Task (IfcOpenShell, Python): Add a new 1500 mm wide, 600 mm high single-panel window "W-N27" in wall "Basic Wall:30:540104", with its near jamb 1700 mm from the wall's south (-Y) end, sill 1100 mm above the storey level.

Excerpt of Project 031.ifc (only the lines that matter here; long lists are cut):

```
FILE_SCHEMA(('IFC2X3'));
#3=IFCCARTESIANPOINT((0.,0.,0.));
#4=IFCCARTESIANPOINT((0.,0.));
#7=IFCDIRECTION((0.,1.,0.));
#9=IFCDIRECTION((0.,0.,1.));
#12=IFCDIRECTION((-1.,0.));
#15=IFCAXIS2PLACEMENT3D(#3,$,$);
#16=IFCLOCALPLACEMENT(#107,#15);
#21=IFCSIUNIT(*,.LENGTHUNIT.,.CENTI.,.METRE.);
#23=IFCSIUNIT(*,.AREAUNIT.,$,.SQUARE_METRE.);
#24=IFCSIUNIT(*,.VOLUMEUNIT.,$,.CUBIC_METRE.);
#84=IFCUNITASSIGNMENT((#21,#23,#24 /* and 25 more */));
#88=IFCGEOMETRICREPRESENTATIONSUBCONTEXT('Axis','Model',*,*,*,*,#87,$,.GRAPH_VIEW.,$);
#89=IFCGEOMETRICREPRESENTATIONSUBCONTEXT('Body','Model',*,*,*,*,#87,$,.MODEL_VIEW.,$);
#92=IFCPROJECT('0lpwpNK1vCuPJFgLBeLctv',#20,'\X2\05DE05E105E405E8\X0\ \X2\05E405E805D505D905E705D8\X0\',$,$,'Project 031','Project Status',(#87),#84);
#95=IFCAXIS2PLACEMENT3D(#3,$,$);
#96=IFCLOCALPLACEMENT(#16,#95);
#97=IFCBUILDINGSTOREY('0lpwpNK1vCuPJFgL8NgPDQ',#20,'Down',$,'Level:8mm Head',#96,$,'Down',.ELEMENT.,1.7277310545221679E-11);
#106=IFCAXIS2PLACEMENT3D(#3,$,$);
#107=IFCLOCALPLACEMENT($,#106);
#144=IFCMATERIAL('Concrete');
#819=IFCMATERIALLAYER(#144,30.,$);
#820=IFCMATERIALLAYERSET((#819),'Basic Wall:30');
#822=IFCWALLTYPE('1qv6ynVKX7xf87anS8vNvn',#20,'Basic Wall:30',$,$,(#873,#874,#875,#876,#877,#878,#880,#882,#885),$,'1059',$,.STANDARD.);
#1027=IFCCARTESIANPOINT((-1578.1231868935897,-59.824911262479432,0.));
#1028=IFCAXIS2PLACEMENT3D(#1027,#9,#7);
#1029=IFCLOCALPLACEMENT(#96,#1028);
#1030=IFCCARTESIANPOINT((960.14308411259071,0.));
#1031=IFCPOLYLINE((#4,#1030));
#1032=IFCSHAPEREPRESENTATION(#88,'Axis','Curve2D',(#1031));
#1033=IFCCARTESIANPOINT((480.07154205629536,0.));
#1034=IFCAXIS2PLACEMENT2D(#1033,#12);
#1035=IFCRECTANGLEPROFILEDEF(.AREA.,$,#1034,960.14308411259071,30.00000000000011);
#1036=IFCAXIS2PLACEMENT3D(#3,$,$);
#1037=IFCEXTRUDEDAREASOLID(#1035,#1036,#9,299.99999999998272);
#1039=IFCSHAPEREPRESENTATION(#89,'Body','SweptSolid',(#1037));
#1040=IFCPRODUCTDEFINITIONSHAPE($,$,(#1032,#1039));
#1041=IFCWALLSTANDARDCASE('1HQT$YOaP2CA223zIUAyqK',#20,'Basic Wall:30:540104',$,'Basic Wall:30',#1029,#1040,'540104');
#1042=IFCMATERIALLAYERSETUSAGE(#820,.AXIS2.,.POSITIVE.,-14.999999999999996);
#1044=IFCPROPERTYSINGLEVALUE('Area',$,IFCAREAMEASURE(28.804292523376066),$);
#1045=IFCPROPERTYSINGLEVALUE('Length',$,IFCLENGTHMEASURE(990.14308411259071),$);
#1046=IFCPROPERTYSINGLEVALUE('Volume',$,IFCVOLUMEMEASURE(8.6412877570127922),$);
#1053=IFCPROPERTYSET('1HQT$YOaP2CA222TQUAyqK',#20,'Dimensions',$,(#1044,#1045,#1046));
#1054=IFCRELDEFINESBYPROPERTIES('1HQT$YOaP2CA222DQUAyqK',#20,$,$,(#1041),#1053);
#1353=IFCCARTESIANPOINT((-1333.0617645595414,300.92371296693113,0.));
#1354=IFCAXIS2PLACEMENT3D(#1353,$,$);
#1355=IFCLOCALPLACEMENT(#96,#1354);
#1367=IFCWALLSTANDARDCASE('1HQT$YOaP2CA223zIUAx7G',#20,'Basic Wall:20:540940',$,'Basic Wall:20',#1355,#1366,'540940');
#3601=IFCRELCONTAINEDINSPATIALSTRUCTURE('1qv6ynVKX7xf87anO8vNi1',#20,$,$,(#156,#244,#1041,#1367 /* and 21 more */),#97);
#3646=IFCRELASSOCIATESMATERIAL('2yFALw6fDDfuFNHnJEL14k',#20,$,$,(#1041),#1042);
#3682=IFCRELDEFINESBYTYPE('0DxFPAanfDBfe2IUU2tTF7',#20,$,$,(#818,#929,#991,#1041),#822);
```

```python
import numpy as np
import ifcopenshell
import ifcopenshell.api.feature
import ifcopenshell.api.geometry
import ifcopenshell.api.pset
import ifcopenshell.api.root
import ifcopenshell.api.spatial
import ifcopenshell.api.type
import ifcopenshell.geom
import ifcopenshell.util.element
import ifcopenshell.util.placement
import ifcopenshell.util.representation
import ifcopenshell.util.shape
import ifcopenshell.util.unit

model = ifcopenshell.open("Project 031.ifc")
unit_scale = ifcopenshell.util.unit.calculate_unit_scale(model)
area_scale = ifcopenshell.util.unit.calculate_unit_scale(model, "AREAUNIT")
volume_scale = ifcopenshell.util.unit.calculate_unit_scale(model, "VOLUMEUNIT")
settings = ifcopenshell.geom.settings()


def volume(element):
    """Net volume in cubic metres, openings subtracted."""
    shape = ifcopenshell.geom.create_shape(settings, element)
    return ifcopenshell.util.shape.get_volume(shape.geometry)


wall = model.by_id(1041)
storey = ifcopenshell.util.element.get_container(wall, ifc_class="IfcBuildingStorey")
context = ifcopenshell.util.representation.get_context(model, "Model", "Body", "MODEL_VIEW")
before = volume(wall)

width, height, from_end, sill = 1.5, 0.6, 1.7, 1.1  # metres

# The wall runs along its own X axis, and the end named is its -X end.
wall_shape = ifcopenshell.geom.create_shape(settings, wall)
x, y, z = ifcopenshell.util.shape.get_vertices(wall_shape.geometry).T
start = x.min() + from_end
face, thickness = float(y.min()), float(y.max() - y.min())
wall_matrix = ifcopenshell.util.placement.get_local_placement(wall.ObjectPlacement)
level = ifcopenshell.util.placement.get_local_placement(storey.ObjectPlacement)[2, 3]


def in_wall(x, y):
    """Placement at x, y metres in the wall's axes, at sill height."""
    matrix = wall_matrix.copy()
    matrix[:, 3] = wall_matrix @ np.array([x / unit_scale, y / unit_scale, 0.0, 1.0])
    matrix[2, 3] = level + sill / unit_scale
    return matrix


# Opening: a box that overshoots both wall faces by 50 mm.
opening = ifcopenshell.api.root.create_entity(model, ifc_class="IfcOpeningElement")
box = ifcopenshell.api.geometry.add_wall_representation(
    model, context=context, length=width, height=height, thickness=thickness + 0.1
)
ifcopenshell.api.geometry.assign_representation(model, product=opening, representation=box)
ifcopenshell.api.geometry.edit_object_placement(model, product=opening, matrix=in_wall(start, face - 0.05), is_si=False)
ifcopenshell.api.feature.add_feature(model, feature=opening, element=wall)

window = ifcopenshell.api.root.create_entity(model, ifc_class="IfcWindow", name="W-N27")
window.OverallWidth, window.OverallHeight = width / unit_scale, height / unit_scale
body = ifcopenshell.api.geometry.add_window_representation(
    model,
    context=context,
    overall_width=window.OverallWidth,
    overall_height=window.OverallHeight,
    partition_type="SINGLE_PANEL",
)
ifcopenshell.api.geometry.assign_representation(model, product=window, representation=body)
ifcopenshell.api.spatial.assign_container(model, products=[window], relating_structure=storey)
fills = ifcopenshell.api.feature.add_filling(model, opening=opening, element=window)
fills.OwnerHistory = window.OwnerHistory  # required in IFC2X3

# IFC2X3 keeps the operation on the window style.
style = ifcopenshell.api.root.create_entity(model, ifc_class="IfcWindowStyle", name="W-N27")
style.OperationType, style.ConstructionType = "SINGLE_PANEL", "NOTDEFINED"
style.ParameterTakesPrecedence = style.Sizeable = False
ifcopenshell.api.type.assign_type(model, related_objects=[window], relating_type=style)

# Centre the window in the wall's thickness.
ifcopenshell.api.geometry.edit_object_placement(model, product=window, matrix=in_wall(start, face), is_si=False)
window_shape = ifcopenshell.geom.create_shape(settings, window)
depth = ifcopenshell.util.shape.get_vertices(window_shape.geometry)[:, 1]
offset = face + thickness / 2 - (depth.min() + depth.max()) / 2
ifcopenshell.api.geometry.edit_object_placement(model, product=window, matrix=in_wall(start, offset), is_si=False)

after = volume(wall)

# Update the wall's stored quantities.
pset = model.by_id(ifcopenshell.util.element.get_pset(wall, "Dimensions", should_inherit=False)["id"])
ifcopenshell.api.pset.edit_pset(model, pset=pset, properties={
    "Area": model.create_entity("IfcAreaMeasure", after / thickness / area_scale),
    "Volume": model.create_entity("IfcVolumeMeasure", after / volume_scale),
})

print(f"wall volume {before:.3f} -> {after:.3f} m3")

model.write("Project 031-out.ifc")
```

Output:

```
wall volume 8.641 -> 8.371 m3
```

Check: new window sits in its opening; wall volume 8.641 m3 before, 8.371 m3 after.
